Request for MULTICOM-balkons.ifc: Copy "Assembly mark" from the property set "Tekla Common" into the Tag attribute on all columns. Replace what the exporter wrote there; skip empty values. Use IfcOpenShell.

First a look at what the model holds.

```python
import ifcopenshell
import ifcopenshell.util.element

model = ifcopenshell.open("MULTICOM-balkons.ifc")
print(model.schema)
columns = model.by_type("IfcColumn")
print(len(columns), "columns")
for e in columns[:8]:
    source = ifcopenshell.util.element.get_pset(e, "Tekla Common", "Assembly mark")
    target = e.Tag
    print(e.id(), repr(source), repr(target), sep=" | ")
```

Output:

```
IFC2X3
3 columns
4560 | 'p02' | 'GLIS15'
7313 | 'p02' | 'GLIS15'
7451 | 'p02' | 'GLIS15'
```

```python
import ifcopenshell
import ifcopenshell.util.element

model = ifcopenshell.open("MULTICOM-balkons.ifc")

count = 0
for e in model.by_type("IfcColumn"):
    value = ifcopenshell.util.element.get_pset(e, "Tekla Common", "Assembly mark")
    current = e.Tag
    if not value or not value.strip() or current == value:
        continue
    e.Tag = value
    count += 1

print(count, "columns updated")

model.write("MULTICOM-balkons_v2.ifc")
```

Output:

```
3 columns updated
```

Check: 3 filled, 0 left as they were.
